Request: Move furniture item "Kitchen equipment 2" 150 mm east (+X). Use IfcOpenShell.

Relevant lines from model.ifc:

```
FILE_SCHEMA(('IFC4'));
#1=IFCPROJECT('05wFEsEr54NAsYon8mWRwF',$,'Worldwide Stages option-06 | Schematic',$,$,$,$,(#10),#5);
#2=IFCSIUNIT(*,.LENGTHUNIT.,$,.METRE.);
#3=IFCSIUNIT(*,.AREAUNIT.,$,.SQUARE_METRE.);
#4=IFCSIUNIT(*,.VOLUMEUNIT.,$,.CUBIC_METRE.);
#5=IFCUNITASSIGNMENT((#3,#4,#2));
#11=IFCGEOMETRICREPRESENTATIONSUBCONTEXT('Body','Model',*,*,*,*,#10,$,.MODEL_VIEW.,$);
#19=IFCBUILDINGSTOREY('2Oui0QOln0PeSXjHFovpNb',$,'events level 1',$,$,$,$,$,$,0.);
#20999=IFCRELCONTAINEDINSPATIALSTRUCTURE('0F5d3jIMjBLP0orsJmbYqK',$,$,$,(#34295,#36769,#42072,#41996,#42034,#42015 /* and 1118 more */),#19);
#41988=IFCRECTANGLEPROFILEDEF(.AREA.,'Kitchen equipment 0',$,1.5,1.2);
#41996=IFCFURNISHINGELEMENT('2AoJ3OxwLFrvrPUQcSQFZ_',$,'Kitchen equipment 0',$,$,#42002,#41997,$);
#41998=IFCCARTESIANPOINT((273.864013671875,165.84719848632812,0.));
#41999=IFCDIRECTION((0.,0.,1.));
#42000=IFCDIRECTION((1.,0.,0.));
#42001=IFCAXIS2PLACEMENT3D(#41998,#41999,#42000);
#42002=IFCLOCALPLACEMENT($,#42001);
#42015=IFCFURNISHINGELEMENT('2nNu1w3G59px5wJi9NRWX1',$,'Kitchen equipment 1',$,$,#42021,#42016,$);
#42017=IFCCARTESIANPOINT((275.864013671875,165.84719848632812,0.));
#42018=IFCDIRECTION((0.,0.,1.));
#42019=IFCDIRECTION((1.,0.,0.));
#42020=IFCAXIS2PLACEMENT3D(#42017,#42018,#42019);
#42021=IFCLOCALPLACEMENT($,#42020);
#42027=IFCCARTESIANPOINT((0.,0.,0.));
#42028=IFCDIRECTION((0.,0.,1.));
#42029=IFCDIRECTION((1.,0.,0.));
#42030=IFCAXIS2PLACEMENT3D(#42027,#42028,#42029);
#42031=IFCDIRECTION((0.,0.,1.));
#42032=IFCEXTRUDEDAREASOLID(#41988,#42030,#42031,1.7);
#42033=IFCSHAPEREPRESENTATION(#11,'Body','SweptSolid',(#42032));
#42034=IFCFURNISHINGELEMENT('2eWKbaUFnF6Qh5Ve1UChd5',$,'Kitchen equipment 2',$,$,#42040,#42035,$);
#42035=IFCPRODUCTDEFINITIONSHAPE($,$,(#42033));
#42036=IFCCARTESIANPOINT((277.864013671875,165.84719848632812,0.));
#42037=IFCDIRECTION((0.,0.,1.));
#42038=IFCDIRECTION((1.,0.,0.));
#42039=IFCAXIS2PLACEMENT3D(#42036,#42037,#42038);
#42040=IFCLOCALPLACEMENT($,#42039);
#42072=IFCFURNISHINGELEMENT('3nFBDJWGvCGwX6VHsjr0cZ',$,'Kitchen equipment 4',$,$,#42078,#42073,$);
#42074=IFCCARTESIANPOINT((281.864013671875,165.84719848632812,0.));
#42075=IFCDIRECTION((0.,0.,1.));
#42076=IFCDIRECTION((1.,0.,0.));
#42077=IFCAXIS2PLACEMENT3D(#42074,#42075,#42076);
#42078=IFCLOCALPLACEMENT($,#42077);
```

```python
import ifcopenshell
import ifcopenshell.api.geometry
import ifcopenshell.util.placement
import ifcopenshell.util.unit

model = ifcopenshell.open("model.ifc")
unit_scale = ifcopenshell.util.unit.calculate_unit_scale(model)

item = model.by_guid("2eWKbaUFnF6Qh5Ve1UChd5")
matrix = ifcopenshell.util.placement.get_local_placement(item.ObjectPlacement)
matrix[0, 3] += 0.15 / unit_scale
ifcopenshell.api.geometry.edit_object_placement(model, product=item, matrix=matrix, is_si=False)

print(ifcopenshell.util.placement.get_local_placement(item.ObjectPlacement).round(3) + 0.0)

model.write("model-out.ifc")
```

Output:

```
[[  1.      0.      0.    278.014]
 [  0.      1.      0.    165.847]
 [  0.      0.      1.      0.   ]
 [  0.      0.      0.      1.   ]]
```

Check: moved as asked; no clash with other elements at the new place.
